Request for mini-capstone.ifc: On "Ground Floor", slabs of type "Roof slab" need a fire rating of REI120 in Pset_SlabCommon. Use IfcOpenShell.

First a look at what the model holds.

```python
import ifcopenshell
import ifcopenshell.util.element

model = ifcopenshell.open("mini-capstone.ifc")
print(model.schema)
storey = next(s for s in model.by_type("IfcBuildingStorey") if s.Name == "Ground Floor")
slabs = [e for e in ifcopenshell.util.element.get_decomposition(storey) if e.is_a("IfcSlab")]
seen = {}
for e in slabs:
    element_type = ifcopenshell.util.element.get_type(e)
    key = (element_type.Name if element_type != e and element_type else None, ifcopenshell.util.element.get_pset(e, "Pset_SlabCommon", "FireRating"))
    seen[key] = seen.get(key, 0) + 1
for (name, value), count in sorted(seen.items(), key=str):
    print(count, "x", name, "|", value)
```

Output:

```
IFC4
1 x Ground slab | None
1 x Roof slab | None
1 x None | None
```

```python
import ifcopenshell
import ifcopenshell.api.pset
import ifcopenshell.util.element

model = ifcopenshell.open("mini-capstone.ifc")

storey = next(s for s in model.by_type("IfcBuildingStorey") if s.Name == "Ground Floor")
slabs = [e for e in ifcopenshell.util.element.get_decomposition(storey) if e.is_a("IfcSlab")]

count = 0
for e in slabs:
    element_type = ifcopenshell.util.element.get_type(e)
    if element_type in (None, e) or element_type.Name != "Roof slab":
        continue
    # add_pset returns the element's existing set when there is one.
    pset = ifcopenshell.api.pset.add_pset(model, product=e, name="Pset_SlabCommon")
    ifcopenshell.api.pset.edit_pset(model, pset=pset, properties={"FireRating": "REI120"})
    count += 1

print(count, "slabs updated")

model.write("mini-capstone_updated.ifc")
```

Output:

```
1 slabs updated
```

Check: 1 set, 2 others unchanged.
